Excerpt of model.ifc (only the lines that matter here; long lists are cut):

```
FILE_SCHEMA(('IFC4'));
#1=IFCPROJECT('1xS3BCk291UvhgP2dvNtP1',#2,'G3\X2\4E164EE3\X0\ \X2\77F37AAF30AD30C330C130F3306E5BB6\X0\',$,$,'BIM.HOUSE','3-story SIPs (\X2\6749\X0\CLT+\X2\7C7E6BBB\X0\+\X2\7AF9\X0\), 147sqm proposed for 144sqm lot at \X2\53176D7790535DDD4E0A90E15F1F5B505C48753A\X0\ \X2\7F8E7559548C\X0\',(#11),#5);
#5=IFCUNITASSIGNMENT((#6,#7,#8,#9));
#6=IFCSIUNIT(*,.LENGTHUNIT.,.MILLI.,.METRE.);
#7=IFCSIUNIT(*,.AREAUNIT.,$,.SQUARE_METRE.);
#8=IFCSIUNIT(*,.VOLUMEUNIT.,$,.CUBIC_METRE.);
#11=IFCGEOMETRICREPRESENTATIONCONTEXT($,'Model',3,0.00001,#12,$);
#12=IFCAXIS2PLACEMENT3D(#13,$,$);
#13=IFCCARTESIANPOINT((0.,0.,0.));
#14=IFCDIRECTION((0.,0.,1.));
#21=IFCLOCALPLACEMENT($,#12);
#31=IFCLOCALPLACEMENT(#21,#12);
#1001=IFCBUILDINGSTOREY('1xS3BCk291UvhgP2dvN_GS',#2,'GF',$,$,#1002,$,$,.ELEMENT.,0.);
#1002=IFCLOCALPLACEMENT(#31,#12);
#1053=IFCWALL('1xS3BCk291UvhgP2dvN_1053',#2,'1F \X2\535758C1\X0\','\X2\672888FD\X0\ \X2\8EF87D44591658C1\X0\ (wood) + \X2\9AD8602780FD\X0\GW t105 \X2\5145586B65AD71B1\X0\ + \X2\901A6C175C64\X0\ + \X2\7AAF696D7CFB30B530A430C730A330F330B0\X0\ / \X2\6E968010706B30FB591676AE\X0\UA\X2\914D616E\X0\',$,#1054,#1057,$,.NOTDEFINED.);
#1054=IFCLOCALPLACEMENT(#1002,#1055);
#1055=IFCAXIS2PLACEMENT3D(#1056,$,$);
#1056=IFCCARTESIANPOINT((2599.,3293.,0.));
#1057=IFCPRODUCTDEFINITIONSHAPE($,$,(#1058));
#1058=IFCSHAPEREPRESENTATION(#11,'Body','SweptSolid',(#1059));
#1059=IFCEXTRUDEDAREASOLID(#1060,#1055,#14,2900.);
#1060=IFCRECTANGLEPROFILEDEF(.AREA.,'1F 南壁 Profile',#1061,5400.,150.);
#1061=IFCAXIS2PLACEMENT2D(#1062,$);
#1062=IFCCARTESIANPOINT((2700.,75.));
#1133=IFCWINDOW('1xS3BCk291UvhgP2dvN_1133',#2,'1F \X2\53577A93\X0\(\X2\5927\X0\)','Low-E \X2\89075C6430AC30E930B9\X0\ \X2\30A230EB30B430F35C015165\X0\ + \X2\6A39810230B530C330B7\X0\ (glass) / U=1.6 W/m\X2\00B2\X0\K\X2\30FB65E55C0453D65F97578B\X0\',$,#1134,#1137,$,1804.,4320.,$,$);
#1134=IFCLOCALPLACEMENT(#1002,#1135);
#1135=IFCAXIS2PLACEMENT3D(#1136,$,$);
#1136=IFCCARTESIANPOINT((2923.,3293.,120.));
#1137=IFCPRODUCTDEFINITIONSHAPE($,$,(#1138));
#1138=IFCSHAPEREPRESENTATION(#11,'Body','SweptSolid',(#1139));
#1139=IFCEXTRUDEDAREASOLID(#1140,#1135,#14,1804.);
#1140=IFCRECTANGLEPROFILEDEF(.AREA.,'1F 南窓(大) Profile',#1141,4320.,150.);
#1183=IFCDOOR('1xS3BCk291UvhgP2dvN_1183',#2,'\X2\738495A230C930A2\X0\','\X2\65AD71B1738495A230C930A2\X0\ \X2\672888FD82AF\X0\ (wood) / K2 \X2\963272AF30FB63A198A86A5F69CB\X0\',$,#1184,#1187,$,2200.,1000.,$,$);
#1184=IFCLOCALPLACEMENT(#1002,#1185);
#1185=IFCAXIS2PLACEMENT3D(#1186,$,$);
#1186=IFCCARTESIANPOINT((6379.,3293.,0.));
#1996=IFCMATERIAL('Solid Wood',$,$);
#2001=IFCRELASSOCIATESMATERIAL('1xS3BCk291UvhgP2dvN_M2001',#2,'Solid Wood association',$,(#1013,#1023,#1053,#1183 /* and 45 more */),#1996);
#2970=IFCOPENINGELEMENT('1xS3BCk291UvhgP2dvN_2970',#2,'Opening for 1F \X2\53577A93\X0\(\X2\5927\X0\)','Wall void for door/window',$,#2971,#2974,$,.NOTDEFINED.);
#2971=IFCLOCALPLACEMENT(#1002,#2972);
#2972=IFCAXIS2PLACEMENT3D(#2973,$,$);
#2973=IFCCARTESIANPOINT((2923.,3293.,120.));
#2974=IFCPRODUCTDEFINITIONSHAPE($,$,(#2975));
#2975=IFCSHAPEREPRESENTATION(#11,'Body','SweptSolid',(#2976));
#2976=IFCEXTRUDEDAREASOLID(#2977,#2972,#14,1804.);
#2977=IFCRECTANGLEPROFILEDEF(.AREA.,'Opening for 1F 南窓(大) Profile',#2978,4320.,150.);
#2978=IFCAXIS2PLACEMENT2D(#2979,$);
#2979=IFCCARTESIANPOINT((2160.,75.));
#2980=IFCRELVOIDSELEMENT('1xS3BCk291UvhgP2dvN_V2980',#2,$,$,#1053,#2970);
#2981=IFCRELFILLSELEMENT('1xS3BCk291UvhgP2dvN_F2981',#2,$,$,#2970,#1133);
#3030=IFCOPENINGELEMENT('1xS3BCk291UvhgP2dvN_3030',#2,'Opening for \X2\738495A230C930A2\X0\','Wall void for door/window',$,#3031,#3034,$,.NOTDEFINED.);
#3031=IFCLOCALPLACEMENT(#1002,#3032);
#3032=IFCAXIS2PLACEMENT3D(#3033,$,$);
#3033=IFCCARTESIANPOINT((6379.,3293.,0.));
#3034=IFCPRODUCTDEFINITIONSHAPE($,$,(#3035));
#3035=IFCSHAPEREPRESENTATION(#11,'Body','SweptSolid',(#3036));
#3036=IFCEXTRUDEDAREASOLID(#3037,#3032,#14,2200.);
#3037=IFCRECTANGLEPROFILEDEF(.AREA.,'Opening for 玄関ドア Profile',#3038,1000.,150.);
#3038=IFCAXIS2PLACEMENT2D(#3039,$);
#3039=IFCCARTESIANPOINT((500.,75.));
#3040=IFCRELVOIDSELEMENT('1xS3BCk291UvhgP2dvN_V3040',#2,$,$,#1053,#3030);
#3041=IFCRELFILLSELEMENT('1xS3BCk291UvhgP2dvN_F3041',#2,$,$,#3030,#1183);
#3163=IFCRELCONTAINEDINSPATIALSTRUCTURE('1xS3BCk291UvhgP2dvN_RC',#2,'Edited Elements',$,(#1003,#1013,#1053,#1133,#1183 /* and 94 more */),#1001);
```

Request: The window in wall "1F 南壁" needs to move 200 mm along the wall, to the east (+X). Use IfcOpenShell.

```python
import ifcopenshell
import ifcopenshell.api.geometry
import ifcopenshell.util.placement
import ifcopenshell.util.unit

model = ifcopenshell.open("model.ifc")
unit_scale = ifcopenshell.util.unit.calculate_unit_scale(model)

window = model.by_id(1133)
opening = window.FillsVoids[0].RelatingOpeningElement
wall = opening.VoidsElements[0].RelatingBuildingElement

wall_matrix = ifcopenshell.util.placement.get_local_placement(wall.ObjectPlacement)
shift = wall_matrix[:3, 0] * 0.2 / unit_scale
before = ifcopenshell.util.placement.get_local_placement(window.ObjectPlacement)[:3, 3].copy()

# The window is not placed relative to its opening, so move both.
for product in (opening, window):
    matrix = ifcopenshell.util.placement.get_local_placement(product.ObjectPlacement)
    matrix[:3, 3] += shift
    ifcopenshell.api.geometry.edit_object_placement(model, product=product, matrix=matrix, is_si=False)

after = ifcopenshell.util.placement.get_local_placement(window.ObjectPlacement)[:3, 3]
print("window moved by", (after - before).round(3) + 0.0)

model.write("model_rev.ifc")
```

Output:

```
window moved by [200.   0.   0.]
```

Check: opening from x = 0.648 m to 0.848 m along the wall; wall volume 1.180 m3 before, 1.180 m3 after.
